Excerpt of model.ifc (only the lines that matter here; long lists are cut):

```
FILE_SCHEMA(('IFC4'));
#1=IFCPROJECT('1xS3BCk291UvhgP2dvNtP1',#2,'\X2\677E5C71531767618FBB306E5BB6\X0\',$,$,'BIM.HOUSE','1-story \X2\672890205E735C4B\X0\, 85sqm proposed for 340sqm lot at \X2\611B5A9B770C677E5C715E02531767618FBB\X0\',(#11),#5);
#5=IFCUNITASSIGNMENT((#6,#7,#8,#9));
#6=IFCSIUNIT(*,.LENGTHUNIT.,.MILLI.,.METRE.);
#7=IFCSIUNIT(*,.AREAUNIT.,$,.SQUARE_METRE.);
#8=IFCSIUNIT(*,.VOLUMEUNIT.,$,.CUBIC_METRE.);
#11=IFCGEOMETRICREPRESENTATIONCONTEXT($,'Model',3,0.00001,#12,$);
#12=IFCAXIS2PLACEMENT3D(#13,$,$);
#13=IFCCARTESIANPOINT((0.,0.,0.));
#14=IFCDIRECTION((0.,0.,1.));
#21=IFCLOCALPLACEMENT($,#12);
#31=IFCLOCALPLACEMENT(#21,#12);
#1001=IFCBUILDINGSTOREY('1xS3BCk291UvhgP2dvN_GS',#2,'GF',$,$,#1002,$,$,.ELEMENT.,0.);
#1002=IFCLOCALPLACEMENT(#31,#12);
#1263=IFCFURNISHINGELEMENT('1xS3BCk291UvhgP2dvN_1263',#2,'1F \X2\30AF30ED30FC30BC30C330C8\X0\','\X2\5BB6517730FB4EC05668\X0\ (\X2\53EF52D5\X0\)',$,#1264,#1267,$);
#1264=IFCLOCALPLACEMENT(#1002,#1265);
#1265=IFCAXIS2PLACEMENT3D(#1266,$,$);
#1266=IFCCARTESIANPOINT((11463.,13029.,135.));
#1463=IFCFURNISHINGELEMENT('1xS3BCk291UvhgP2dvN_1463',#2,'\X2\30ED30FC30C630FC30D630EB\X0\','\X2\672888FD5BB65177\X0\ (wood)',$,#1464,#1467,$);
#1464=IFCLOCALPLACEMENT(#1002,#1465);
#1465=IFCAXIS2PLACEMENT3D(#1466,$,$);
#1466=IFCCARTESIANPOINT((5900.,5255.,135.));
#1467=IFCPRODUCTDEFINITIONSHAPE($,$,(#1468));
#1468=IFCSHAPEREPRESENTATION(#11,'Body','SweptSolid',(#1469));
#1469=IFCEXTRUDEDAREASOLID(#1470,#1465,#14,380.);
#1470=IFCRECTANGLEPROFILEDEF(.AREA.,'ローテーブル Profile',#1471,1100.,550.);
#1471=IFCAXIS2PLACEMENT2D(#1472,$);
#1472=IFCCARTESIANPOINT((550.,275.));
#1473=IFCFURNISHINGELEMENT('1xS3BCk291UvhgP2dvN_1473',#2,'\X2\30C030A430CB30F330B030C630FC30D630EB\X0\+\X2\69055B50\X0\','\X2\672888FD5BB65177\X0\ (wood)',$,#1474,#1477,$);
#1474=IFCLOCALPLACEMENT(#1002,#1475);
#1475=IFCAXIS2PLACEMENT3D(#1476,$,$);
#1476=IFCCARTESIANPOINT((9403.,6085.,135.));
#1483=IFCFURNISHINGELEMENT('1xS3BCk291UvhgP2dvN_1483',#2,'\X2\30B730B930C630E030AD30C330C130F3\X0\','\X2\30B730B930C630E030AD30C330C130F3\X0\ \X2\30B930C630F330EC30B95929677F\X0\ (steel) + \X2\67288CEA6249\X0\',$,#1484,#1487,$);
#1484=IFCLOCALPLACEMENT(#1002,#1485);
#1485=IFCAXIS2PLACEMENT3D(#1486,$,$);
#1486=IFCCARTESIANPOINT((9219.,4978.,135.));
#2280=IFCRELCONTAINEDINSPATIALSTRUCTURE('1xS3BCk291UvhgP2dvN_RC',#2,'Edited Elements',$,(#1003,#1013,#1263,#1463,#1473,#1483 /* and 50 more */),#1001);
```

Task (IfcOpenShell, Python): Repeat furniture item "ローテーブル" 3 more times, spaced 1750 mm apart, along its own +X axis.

```python
import ifcopenshell
import ifcopenshell.api.geometry
import ifcopenshell.api.root
import ifcopenshell.util.element
import ifcopenshell.util.placement

model = ifcopenshell.open("model.ifc")


def reuse_history(source, copy):
    """copy_class also copies each property set's owner history, people and application; keep the originals."""
    for rel in copy.IsDefinedBy:
        if rel.is_a("IfcRelDefinesByProperties") and (history := rel.RelatingPropertyDefinition.OwnerHistory):
            rel.RelatingPropertyDefinition.OwnerHistory = source.OwnerHistory
            ifcopenshell.util.element.remove_deep2(model, history)


source = model.by_guid("1xS3BCk291UvhgP2dvN_1463")
base = ifcopenshell.util.placement.get_local_placement(source.ObjectPlacement)
step = base[:3, 0] * 1750.0

for i in range(1, 4):
    copy = ifcopenshell.api.root.copy_class(model, product=source)
    copy.Representation = ifcopenshell.util.element.copy_deep(
        model, source.Representation, exclude=["IfcGeometricRepresentationContext", "IfcRepresentationMap"]
    )
    reuse_history(source, copy)
    matrix = base.copy()
    matrix[:3, 3] += i * step
    print("added at", matrix[:3, 3].round(3) + 0.0)
    ifcopenshell.api.geometry.edit_object_placement(model, product=copy, matrix=matrix, is_si=False)

model.write("model_v2.ifc")
```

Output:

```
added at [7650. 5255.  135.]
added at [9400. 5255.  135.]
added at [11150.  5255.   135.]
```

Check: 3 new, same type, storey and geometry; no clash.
